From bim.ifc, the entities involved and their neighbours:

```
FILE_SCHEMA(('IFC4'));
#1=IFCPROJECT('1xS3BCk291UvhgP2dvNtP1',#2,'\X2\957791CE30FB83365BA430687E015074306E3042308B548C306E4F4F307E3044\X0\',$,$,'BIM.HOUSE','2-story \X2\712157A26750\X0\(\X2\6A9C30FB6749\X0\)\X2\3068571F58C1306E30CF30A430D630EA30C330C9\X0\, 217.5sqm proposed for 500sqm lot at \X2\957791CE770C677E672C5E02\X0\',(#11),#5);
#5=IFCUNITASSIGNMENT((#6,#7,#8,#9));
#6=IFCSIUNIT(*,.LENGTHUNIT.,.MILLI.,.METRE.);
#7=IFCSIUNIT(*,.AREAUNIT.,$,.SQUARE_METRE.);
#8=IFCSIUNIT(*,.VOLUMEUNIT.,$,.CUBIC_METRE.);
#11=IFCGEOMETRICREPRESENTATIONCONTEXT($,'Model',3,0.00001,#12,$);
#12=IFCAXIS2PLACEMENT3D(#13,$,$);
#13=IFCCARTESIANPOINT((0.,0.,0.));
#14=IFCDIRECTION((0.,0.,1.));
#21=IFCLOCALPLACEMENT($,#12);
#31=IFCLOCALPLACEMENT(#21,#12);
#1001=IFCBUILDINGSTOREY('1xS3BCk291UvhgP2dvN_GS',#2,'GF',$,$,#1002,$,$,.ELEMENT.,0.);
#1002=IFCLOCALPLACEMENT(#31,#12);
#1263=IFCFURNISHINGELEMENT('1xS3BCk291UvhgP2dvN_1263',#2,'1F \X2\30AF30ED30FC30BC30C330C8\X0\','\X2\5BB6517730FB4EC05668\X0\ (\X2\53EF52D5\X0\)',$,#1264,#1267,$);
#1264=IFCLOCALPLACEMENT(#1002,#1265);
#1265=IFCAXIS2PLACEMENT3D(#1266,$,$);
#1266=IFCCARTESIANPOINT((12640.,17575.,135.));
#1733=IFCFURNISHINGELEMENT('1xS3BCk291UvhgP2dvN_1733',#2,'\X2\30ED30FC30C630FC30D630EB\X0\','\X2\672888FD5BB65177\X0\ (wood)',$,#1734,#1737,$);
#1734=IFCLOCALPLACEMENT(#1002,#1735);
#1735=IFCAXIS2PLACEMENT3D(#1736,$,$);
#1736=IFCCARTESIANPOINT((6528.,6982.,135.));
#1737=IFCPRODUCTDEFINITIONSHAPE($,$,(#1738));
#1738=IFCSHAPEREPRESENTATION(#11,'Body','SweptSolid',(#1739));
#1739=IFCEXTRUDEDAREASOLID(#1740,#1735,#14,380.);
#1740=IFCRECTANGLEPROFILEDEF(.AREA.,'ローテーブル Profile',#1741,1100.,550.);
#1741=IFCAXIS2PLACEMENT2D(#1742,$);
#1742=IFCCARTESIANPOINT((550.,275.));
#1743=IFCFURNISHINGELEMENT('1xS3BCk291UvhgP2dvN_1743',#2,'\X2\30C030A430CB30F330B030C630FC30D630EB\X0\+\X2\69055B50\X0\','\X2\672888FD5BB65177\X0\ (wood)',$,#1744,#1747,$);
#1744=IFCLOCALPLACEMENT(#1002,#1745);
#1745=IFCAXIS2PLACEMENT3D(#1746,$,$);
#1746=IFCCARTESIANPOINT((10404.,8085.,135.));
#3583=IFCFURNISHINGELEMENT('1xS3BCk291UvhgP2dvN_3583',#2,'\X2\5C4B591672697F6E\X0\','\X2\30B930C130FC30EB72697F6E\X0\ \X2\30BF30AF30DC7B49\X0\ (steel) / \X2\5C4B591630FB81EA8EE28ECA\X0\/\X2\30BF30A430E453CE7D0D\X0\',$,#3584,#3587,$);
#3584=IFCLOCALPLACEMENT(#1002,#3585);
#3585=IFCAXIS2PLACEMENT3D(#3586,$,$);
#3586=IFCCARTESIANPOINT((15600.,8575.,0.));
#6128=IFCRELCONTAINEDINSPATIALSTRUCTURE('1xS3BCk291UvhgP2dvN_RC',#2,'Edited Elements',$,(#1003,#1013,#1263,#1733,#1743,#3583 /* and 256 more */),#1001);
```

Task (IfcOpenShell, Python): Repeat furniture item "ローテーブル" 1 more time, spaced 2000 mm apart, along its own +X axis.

```python
import ifcopenshell
import ifcopenshell.api.geometry
import ifcopenshell.api.root
import ifcopenshell.util.element
import ifcopenshell.util.placement
import ifcopenshell.util.unit

model = ifcopenshell.open("bim.ifc")
unit_scale = ifcopenshell.util.unit.calculate_unit_scale(model)


def reuse_history(source, copy):
    """copy_class also copies each property set's owner history, people and application; keep the originals."""
    for rel in copy.IsDefinedBy:
        if rel.is_a("IfcRelDefinesByProperties") and (history := rel.RelatingPropertyDefinition.OwnerHistory):
            rel.RelatingPropertyDefinition.OwnerHistory = source.OwnerHistory
            ifcopenshell.util.element.remove_deep2(model, history)


source = model.by_guid("1xS3BCk291UvhgP2dvN_1733")
base = ifcopenshell.util.placement.get_local_placement(source.ObjectPlacement)
step = base[:3, 0] * 2 / unit_scale

for i in range(1, 2):
    copy = ifcopenshell.api.root.copy_class(model, product=source)
    copy.Representation = ifcopenshell.util.element.copy_deep(
        model, source.Representation, exclude=["IfcGeometricRepresentationContext", "IfcRepresentationMap"]
    )
    reuse_history(source, copy)
    matrix = base.copy()
    matrix[:3, 3] += i * step
    print("added at", matrix[:3, 3].round(3) + 0.0)
    ifcopenshell.api.geometry.edit_object_placement(model, product=copy, matrix=matrix, is_si=False)

model.write("bim_edited.ifc")
```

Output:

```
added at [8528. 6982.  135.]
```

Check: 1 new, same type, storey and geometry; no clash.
